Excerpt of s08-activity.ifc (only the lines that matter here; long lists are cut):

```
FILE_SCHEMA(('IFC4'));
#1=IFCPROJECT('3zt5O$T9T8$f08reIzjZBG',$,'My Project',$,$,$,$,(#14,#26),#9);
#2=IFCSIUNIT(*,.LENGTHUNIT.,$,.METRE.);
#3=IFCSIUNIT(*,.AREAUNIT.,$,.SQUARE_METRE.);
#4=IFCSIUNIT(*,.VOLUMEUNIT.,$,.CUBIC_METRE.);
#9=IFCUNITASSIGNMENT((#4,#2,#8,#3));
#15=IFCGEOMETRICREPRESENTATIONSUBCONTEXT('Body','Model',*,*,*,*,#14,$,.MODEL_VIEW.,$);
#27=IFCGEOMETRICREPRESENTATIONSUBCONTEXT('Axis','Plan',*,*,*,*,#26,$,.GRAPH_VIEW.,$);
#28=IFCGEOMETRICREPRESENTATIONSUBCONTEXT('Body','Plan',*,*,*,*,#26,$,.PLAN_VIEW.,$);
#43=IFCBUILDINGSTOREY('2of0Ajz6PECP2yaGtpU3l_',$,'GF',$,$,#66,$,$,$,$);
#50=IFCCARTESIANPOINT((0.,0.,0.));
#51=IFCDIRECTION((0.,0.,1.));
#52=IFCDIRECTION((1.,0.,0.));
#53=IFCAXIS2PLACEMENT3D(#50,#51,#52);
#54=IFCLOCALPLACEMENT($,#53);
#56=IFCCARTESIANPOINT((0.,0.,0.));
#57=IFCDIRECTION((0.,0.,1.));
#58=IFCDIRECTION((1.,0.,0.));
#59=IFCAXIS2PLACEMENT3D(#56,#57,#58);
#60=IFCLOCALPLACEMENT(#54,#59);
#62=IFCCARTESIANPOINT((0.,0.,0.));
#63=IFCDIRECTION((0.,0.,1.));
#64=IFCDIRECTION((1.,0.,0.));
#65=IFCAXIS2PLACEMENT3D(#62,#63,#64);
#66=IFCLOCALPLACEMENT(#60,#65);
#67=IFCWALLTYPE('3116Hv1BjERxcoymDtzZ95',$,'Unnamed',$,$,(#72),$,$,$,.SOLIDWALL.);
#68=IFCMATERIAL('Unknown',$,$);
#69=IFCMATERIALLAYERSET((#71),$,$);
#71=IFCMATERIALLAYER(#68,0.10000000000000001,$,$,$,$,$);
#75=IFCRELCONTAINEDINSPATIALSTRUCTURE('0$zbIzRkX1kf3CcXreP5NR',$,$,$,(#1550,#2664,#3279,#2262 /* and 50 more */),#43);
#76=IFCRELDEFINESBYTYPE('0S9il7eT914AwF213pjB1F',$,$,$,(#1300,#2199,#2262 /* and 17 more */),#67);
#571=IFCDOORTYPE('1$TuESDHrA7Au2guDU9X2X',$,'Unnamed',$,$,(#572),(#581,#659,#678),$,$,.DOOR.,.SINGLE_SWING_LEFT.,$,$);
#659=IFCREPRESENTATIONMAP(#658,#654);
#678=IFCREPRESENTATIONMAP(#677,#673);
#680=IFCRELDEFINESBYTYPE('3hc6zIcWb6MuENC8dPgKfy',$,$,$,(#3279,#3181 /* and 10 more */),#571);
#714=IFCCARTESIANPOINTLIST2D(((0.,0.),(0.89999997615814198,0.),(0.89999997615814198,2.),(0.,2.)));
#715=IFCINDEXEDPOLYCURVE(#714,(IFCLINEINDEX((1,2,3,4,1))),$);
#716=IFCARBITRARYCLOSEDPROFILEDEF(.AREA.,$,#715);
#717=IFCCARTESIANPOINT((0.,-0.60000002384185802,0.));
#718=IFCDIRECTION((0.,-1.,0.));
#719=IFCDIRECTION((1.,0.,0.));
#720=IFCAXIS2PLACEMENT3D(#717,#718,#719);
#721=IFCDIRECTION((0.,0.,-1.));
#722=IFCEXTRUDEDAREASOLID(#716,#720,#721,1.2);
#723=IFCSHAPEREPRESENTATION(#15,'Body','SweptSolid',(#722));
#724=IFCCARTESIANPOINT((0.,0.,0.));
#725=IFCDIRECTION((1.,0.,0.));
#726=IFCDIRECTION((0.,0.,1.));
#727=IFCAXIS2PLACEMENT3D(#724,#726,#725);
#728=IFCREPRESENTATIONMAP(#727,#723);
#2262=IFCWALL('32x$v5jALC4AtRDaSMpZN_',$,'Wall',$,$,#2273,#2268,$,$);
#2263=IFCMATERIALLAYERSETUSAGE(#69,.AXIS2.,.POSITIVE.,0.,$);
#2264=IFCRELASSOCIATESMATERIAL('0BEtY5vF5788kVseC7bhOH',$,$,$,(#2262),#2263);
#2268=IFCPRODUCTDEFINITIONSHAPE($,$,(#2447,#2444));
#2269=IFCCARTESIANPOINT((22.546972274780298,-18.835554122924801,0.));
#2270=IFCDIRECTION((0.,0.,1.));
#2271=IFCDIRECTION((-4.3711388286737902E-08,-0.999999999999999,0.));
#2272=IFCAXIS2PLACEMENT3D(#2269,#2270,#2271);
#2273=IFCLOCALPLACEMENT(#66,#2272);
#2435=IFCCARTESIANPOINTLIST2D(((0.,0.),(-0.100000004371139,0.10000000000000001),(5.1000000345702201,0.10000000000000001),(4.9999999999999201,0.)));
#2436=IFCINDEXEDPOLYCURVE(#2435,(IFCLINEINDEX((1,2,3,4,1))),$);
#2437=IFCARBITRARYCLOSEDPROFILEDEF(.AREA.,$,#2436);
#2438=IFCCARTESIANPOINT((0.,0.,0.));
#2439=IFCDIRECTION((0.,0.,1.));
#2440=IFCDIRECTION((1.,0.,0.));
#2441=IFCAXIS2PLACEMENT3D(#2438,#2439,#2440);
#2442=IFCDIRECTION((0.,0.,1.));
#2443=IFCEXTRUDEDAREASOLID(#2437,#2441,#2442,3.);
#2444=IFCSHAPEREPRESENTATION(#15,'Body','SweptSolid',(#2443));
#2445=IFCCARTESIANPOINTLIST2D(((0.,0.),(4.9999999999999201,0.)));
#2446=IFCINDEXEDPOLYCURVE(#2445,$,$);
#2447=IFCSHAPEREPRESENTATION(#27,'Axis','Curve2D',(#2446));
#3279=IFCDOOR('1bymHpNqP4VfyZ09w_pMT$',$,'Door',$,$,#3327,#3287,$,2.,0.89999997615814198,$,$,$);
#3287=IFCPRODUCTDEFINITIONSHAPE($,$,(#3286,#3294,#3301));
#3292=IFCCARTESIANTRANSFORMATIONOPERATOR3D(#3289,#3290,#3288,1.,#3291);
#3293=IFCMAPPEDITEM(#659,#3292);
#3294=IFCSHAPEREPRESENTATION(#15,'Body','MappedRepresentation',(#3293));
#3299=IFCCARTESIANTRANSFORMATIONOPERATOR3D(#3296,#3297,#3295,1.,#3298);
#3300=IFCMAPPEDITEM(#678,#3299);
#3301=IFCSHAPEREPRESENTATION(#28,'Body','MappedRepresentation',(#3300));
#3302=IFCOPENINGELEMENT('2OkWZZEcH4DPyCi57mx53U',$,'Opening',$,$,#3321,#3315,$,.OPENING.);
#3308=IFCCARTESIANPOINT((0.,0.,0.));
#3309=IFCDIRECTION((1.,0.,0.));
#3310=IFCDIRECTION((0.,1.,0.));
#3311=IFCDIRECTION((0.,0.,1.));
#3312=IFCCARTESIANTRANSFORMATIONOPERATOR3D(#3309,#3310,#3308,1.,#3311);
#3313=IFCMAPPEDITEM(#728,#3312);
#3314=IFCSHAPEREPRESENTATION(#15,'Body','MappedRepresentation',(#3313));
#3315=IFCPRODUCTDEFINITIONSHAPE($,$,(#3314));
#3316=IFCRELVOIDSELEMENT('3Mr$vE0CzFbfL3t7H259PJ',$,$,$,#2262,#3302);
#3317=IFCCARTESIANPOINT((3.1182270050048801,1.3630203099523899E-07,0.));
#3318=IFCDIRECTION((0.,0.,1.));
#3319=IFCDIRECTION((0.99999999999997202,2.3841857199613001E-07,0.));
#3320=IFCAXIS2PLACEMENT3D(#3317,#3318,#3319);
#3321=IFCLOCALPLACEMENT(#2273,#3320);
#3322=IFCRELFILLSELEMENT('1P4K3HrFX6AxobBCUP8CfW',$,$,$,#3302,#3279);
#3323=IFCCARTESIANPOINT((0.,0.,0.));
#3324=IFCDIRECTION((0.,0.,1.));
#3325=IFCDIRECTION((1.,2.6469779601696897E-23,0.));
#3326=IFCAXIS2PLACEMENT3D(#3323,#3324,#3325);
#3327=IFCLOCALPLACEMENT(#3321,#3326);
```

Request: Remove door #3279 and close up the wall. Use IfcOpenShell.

```python
import ifcopenshell
import ifcopenshell.api.feature
import ifcopenshell.api.root
import ifcopenshell.geom
import ifcopenshell.util.shape

model = ifcopenshell.open("s08-activity.ifc")
settings = ifcopenshell.geom.settings()


def volume(element):
    """Net volume in cubic metres, openings subtracted."""
    shape = ifcopenshell.geom.create_shape(settings, element)
    return ifcopenshell.util.shape.get_volume(shape.geometry)


door = model.by_id(3279)
opening = door.FillsVoids[0].RelatingOpeningElement
wall = opening.VoidsElements[0].RelatingBuildingElement
before = volume(wall)

ifcopenshell.api.root.remove_product(model, product=door)
ifcopenshell.api.feature.remove_feature(model, feature=opening)

after = volume(wall)

print(f"wall volume {before:.3f} -> {after:.3f} m3")

model.write("s08-activity-out.ifc")
```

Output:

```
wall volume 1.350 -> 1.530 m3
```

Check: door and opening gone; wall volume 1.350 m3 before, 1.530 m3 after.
